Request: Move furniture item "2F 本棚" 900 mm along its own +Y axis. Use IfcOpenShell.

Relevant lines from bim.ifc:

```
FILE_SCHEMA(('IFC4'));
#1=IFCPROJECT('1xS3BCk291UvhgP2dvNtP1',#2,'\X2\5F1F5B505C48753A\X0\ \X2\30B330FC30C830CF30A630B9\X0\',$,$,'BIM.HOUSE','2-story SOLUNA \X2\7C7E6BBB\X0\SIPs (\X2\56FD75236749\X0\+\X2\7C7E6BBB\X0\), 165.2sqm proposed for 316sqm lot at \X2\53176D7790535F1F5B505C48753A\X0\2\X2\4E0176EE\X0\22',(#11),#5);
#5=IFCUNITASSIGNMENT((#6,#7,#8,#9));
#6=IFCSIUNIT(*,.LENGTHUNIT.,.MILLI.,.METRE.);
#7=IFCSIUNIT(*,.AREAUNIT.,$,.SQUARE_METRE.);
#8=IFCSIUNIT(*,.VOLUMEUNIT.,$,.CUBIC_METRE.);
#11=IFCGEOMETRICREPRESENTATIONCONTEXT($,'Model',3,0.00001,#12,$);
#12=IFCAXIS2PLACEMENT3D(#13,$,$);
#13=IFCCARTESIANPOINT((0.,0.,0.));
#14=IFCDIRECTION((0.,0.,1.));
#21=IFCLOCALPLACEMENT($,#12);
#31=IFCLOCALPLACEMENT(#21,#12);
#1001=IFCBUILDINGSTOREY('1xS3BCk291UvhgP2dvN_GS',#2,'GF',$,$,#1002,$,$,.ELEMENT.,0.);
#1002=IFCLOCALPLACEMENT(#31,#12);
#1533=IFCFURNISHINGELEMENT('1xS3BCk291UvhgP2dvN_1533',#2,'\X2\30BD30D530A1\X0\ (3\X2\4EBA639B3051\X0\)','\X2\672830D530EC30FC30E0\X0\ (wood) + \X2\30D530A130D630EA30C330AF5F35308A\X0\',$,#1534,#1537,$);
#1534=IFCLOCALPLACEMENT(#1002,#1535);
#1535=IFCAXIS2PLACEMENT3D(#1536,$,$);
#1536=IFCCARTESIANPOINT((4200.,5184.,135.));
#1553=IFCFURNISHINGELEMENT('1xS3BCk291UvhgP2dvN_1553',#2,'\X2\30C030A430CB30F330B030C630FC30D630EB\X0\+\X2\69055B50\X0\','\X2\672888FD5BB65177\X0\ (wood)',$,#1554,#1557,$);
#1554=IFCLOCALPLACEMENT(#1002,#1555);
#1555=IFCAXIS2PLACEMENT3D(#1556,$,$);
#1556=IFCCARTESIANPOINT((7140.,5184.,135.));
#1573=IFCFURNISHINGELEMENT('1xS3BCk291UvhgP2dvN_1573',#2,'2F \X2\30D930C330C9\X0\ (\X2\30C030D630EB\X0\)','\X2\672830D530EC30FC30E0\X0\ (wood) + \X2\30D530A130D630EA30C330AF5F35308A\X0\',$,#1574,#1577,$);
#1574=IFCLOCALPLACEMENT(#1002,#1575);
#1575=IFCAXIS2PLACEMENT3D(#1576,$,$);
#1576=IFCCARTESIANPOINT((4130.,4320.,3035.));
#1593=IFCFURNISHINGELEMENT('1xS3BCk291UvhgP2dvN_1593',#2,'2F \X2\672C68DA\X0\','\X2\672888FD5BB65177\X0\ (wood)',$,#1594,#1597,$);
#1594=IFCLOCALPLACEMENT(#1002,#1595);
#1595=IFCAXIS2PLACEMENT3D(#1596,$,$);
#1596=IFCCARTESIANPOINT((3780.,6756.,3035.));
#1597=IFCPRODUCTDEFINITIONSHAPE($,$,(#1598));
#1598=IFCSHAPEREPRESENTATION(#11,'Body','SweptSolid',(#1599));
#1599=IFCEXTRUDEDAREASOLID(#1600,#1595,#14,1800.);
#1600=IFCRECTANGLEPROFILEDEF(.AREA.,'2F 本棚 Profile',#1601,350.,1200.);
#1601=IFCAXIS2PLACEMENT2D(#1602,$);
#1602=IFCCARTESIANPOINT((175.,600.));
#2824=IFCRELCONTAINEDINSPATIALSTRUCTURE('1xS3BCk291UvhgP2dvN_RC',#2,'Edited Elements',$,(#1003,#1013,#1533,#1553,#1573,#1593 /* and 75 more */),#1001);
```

```python
import ifcopenshell
import ifcopenshell.api.geometry
import ifcopenshell.util.placement
import ifcopenshell.util.unit

model = ifcopenshell.open("bim.ifc")
unit_scale = ifcopenshell.util.unit.calculate_unit_scale(model)

item = model.by_guid("1xS3BCk291UvhgP2dvN_1593")
matrix = ifcopenshell.util.placement.get_local_placement(item.ObjectPlacement)
matrix[:3, 3] += matrix[:3, 1] * 0.9 / unit_scale
ifcopenshell.api.geometry.edit_object_placement(model, product=item, matrix=matrix, is_si=False)

print(ifcopenshell.util.placement.get_local_placement(item.ObjectPlacement).round(3) + 0.0)

model.write("bim_updated.ifc")
```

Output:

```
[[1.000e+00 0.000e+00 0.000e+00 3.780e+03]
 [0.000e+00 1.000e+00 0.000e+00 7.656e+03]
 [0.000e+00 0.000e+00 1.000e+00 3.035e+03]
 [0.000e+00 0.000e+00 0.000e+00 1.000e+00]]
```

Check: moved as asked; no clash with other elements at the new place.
